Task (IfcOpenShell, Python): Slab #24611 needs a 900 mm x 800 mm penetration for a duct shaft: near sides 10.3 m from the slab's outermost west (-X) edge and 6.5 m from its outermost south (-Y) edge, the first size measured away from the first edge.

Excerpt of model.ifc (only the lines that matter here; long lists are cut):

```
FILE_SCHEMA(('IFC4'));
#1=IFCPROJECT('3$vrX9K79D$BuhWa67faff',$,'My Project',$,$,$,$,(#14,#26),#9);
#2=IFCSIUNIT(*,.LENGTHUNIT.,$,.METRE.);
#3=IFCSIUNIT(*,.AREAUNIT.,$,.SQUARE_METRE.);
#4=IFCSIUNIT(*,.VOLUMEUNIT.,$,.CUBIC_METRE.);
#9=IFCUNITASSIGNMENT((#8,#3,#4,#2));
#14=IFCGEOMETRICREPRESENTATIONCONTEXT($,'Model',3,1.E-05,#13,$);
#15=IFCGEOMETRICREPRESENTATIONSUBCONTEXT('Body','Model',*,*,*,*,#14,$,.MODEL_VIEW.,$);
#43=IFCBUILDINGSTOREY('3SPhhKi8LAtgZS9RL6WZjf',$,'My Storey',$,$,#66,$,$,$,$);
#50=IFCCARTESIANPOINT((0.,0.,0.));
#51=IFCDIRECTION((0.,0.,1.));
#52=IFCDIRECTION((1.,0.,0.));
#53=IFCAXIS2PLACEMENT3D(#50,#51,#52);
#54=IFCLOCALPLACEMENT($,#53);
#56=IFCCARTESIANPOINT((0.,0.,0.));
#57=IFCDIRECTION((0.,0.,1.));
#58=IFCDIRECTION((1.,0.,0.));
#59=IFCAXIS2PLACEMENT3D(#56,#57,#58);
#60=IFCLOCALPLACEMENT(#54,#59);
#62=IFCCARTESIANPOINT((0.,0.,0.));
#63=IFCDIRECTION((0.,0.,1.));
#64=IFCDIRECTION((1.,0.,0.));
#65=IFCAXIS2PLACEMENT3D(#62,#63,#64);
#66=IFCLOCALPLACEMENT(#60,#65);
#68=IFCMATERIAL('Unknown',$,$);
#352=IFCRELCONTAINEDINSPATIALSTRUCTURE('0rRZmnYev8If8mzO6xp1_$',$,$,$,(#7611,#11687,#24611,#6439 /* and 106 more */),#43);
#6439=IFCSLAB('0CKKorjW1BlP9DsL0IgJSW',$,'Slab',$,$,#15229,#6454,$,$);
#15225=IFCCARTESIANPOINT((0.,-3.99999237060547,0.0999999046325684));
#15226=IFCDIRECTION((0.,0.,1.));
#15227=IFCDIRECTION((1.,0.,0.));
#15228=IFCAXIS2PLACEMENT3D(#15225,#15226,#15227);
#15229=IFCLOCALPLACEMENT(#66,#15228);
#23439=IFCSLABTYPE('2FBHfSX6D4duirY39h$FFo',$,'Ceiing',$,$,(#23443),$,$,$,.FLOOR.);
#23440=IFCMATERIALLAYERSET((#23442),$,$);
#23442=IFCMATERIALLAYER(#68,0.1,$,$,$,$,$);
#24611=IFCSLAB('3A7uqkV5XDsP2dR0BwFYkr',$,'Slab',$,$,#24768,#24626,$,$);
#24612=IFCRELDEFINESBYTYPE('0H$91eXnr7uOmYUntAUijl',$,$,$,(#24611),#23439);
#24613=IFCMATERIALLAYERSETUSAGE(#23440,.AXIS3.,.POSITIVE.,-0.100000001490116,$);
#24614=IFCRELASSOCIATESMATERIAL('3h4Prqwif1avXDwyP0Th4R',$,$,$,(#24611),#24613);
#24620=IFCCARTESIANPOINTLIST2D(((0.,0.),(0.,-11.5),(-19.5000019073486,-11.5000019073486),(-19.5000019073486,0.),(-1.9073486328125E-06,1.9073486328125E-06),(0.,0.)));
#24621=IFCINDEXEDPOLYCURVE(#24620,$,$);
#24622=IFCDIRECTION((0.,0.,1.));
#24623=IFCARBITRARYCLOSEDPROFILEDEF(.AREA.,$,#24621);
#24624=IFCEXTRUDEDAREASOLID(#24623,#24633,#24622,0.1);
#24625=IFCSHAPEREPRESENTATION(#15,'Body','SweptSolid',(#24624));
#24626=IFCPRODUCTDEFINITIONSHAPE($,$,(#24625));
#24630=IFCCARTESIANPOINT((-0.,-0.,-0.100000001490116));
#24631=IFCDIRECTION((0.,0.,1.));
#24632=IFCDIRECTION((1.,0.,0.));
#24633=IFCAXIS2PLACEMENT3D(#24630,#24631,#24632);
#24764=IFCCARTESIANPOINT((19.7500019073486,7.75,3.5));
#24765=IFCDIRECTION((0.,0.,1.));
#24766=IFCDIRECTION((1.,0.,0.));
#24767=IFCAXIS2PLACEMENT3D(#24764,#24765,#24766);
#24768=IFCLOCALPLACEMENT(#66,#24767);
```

```python
import numpy as np
import ifcopenshell
import ifcopenshell.api.feature
import ifcopenshell.api.geometry
import ifcopenshell.api.root
import ifcopenshell.geom
import ifcopenshell.util.placement
import ifcopenshell.util.representation
import ifcopenshell.util.shape
import ifcopenshell.util.unit

model = ifcopenshell.open("model.ifc")
unit_scale = ifcopenshell.util.unit.calculate_unit_scale(model)
settings = ifcopenshell.geom.settings()


def volume(element):
    """Net volume in cubic metres, openings subtracted."""
    shape = ifcopenshell.geom.create_shape(settings, element)
    return ifcopenshell.util.shape.get_volume(shape.geometry)


slab = model.by_guid("3A7uqkV5XDsP2dR0BwFYkr")
before = volume(slab)

# Extent in the slab's own axes, in metres. The edges named are its -X and -Y sides.
slab_shape = ifcopenshell.geom.create_shape(settings, slab)
vertices = ifcopenshell.util.shape.get_vertices(slab_shape.geometry)
x_min, y_min, bottom = vertices.min(axis=0)
top = vertices[:, 2].max()

opening = ifcopenshell.api.root.create_entity(model, ifc_class="IfcOpeningElement", name="Duct shaft opening", predefined_type="OPENING")
context = ifcopenshell.util.representation.get_context(model, "Model", "Body", "MODEL_VIEW")
width, depth = 0.9, 0.8
outline = [(0.0, 0.0), (width, 0.0), (width, depth), (0.0, depth), (0.0, 0.0)]
# Overshoot both faces by 50 mm so the cut is clean.
shape = ifcopenshell.api.geometry.add_slab_representation(
    model, context=context, depth=top - bottom + 0.1, polyline=outline
)
ifcopenshell.api.geometry.assign_representation(model, product=opening, representation=shape)

matrix = ifcopenshell.util.placement.get_local_placement(slab.ObjectPlacement)
matrix[:, 3] = matrix @ np.append(np.array([x_min + 10.3, y_min + 6.5, bottom - 0.05]) / unit_scale, 1.0)
ifcopenshell.api.geometry.edit_object_placement(model, product=opening, matrix=matrix, is_si=False)
ifcopenshell.api.feature.add_feature(model, feature=opening, element=slab)

after = volume(slab)

print(f"slab volume {before:.3f} -> {after:.3f} m3")

model.write("model_edited.ifc")
```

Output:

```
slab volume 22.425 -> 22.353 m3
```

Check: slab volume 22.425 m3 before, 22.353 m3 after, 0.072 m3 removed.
